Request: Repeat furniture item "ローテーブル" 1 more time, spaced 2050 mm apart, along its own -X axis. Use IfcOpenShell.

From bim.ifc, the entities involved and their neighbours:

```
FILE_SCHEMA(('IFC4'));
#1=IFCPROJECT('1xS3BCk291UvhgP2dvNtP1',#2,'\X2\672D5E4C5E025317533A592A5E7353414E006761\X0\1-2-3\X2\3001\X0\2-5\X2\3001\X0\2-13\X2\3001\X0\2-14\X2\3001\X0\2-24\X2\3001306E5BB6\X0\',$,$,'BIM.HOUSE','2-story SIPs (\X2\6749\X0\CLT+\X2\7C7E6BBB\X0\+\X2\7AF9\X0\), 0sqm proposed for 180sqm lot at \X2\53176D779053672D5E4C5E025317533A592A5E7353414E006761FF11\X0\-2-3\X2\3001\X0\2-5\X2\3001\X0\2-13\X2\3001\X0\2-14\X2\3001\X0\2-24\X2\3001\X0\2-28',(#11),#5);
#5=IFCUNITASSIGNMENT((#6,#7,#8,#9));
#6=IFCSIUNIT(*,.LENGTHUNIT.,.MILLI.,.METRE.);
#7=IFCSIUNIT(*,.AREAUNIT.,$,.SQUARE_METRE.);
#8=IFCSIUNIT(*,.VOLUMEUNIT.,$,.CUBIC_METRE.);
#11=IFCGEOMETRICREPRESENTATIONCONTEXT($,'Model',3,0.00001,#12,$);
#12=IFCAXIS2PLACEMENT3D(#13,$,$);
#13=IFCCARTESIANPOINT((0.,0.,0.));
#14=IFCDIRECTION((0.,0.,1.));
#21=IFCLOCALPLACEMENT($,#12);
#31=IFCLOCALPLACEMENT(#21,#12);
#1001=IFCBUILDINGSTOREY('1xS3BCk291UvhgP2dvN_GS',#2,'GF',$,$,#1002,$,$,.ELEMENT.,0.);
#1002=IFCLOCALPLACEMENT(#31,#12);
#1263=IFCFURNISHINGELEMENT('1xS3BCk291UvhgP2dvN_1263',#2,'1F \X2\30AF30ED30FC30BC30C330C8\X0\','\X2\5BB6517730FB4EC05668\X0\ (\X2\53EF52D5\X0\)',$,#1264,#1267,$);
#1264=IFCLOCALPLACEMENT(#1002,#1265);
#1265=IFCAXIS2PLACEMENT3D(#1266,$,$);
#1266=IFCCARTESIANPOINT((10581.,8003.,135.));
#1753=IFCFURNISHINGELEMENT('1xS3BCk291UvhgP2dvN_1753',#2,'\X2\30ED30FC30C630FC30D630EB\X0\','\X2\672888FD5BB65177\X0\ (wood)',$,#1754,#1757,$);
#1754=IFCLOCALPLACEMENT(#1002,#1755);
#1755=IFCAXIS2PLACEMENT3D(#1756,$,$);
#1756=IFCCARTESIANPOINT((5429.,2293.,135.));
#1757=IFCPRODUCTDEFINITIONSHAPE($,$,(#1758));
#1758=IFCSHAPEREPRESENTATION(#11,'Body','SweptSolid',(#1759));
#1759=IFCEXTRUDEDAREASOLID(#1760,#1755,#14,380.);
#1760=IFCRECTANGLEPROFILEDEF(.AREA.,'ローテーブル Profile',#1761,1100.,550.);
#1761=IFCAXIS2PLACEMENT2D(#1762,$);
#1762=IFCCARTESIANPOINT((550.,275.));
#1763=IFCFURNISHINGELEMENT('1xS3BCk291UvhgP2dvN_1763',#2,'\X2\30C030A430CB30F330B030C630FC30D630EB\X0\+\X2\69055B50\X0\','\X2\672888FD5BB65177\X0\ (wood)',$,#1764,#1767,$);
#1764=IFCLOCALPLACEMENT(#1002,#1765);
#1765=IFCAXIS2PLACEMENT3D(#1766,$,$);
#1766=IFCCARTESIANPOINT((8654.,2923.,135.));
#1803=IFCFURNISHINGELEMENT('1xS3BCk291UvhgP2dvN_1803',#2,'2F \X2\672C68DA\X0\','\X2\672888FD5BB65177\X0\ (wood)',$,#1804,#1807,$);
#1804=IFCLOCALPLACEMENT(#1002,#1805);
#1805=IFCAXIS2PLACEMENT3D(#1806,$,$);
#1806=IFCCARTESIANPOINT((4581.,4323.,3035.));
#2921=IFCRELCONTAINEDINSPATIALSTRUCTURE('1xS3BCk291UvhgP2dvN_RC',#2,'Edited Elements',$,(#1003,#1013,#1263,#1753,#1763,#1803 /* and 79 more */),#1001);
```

```python
import ifcopenshell
import ifcopenshell.api.geometry
import ifcopenshell.api.root
import ifcopenshell.util.element
import ifcopenshell.util.placement

model = ifcopenshell.open("bim.ifc")


def reuse_history(source, copy):
    """copy_class also copies each property set's owner history, people and application; keep the originals."""
    for rel in copy.IsDefinedBy:
        if rel.is_a("IfcRelDefinesByProperties") and (history := rel.RelatingPropertyDefinition.OwnerHistory):
            rel.RelatingPropertyDefinition.OwnerHistory = source.OwnerHistory
            ifcopenshell.util.element.remove_deep2(model, history)


source = model.by_guid("1xS3BCk291UvhgP2dvN_1753")
base = ifcopenshell.util.placement.get_local_placement(source.ObjectPlacement)
step = -base[:3, 0] * 2050.0

for i in range(1, 2):
    copy = ifcopenshell.api.root.copy_class(model, product=source)
    copy.Representation = ifcopenshell.util.element.copy_deep(
        model, source.Representation, exclude=["IfcGeometricRepresentationContext", "IfcRepresentationMap"]
    )
    reuse_history(source, copy)
    matrix = base.copy()
    matrix[:3, 3] += i * step
    print("added at", matrix[:3, 3].round(3) + 0.0)
    ifcopenshell.api.geometry.edit_object_placement(model, product=copy, matrix=matrix, is_si=False)

model.write("bim_v2.ifc")
```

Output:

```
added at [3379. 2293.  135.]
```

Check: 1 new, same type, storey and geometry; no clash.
